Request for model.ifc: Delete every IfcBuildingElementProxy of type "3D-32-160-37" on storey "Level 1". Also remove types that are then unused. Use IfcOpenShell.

First a look at what the model holds.

```python
import ifcopenshell
import ifcopenshell.util.element

model = ifcopenshell.open("model.ifc")
print(model.schema)
storey = next(s for s in model.by_type("IfcBuildingStorey") if s.Name == "Level 1")
proxies = [e for e in ifcopenshell.util.element.get_decomposition(storey) if e.is_a("IfcBuildingElementProxy")]
seen = {}
for e in proxies:
    element_type = ifcopenshell.util.element.get_type(e)
    name = element_type.Name if element_type not in (None, e) else None
    seen[name] = seen.get(name, 0) + 1
for name, count in sorted(seen.items(), key=str):
    print(count, "x", name)
```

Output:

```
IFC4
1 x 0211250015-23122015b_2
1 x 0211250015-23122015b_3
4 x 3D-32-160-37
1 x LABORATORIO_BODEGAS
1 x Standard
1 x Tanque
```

```python
import ifcopenshell
import ifcopenshell.api.root
import ifcopenshell.util.element

model = ifcopenshell.open("model.ifc")

storey = next(s for s in model.by_type("IfcBuildingStorey") if s.Name == "Level 1")
proxies = [e for e in ifcopenshell.util.element.get_decomposition(storey) if e.is_a("IfcBuildingElementProxy")]
targets = [e for e in proxies if (t := ifcopenshell.util.element.get_type(e)) not in (None, e) and t.Name == "3D-32-160-37"]
types = {ifcopenshell.util.element.get_type(e) for e in targets} - {None, *targets}

for e in targets:
    ifcopenshell.api.root.remove_product(model, product=e)
print(len(targets), "removed")

unused = [t for t in types if not ifcopenshell.util.element.get_types(t)]
for t in unused:
    ifcopenshell.api.root.remove_product(model, product=t)
print(len(unused), "unused types removed")

model.write("model_updated.ifc")
```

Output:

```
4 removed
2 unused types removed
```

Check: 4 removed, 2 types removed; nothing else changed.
